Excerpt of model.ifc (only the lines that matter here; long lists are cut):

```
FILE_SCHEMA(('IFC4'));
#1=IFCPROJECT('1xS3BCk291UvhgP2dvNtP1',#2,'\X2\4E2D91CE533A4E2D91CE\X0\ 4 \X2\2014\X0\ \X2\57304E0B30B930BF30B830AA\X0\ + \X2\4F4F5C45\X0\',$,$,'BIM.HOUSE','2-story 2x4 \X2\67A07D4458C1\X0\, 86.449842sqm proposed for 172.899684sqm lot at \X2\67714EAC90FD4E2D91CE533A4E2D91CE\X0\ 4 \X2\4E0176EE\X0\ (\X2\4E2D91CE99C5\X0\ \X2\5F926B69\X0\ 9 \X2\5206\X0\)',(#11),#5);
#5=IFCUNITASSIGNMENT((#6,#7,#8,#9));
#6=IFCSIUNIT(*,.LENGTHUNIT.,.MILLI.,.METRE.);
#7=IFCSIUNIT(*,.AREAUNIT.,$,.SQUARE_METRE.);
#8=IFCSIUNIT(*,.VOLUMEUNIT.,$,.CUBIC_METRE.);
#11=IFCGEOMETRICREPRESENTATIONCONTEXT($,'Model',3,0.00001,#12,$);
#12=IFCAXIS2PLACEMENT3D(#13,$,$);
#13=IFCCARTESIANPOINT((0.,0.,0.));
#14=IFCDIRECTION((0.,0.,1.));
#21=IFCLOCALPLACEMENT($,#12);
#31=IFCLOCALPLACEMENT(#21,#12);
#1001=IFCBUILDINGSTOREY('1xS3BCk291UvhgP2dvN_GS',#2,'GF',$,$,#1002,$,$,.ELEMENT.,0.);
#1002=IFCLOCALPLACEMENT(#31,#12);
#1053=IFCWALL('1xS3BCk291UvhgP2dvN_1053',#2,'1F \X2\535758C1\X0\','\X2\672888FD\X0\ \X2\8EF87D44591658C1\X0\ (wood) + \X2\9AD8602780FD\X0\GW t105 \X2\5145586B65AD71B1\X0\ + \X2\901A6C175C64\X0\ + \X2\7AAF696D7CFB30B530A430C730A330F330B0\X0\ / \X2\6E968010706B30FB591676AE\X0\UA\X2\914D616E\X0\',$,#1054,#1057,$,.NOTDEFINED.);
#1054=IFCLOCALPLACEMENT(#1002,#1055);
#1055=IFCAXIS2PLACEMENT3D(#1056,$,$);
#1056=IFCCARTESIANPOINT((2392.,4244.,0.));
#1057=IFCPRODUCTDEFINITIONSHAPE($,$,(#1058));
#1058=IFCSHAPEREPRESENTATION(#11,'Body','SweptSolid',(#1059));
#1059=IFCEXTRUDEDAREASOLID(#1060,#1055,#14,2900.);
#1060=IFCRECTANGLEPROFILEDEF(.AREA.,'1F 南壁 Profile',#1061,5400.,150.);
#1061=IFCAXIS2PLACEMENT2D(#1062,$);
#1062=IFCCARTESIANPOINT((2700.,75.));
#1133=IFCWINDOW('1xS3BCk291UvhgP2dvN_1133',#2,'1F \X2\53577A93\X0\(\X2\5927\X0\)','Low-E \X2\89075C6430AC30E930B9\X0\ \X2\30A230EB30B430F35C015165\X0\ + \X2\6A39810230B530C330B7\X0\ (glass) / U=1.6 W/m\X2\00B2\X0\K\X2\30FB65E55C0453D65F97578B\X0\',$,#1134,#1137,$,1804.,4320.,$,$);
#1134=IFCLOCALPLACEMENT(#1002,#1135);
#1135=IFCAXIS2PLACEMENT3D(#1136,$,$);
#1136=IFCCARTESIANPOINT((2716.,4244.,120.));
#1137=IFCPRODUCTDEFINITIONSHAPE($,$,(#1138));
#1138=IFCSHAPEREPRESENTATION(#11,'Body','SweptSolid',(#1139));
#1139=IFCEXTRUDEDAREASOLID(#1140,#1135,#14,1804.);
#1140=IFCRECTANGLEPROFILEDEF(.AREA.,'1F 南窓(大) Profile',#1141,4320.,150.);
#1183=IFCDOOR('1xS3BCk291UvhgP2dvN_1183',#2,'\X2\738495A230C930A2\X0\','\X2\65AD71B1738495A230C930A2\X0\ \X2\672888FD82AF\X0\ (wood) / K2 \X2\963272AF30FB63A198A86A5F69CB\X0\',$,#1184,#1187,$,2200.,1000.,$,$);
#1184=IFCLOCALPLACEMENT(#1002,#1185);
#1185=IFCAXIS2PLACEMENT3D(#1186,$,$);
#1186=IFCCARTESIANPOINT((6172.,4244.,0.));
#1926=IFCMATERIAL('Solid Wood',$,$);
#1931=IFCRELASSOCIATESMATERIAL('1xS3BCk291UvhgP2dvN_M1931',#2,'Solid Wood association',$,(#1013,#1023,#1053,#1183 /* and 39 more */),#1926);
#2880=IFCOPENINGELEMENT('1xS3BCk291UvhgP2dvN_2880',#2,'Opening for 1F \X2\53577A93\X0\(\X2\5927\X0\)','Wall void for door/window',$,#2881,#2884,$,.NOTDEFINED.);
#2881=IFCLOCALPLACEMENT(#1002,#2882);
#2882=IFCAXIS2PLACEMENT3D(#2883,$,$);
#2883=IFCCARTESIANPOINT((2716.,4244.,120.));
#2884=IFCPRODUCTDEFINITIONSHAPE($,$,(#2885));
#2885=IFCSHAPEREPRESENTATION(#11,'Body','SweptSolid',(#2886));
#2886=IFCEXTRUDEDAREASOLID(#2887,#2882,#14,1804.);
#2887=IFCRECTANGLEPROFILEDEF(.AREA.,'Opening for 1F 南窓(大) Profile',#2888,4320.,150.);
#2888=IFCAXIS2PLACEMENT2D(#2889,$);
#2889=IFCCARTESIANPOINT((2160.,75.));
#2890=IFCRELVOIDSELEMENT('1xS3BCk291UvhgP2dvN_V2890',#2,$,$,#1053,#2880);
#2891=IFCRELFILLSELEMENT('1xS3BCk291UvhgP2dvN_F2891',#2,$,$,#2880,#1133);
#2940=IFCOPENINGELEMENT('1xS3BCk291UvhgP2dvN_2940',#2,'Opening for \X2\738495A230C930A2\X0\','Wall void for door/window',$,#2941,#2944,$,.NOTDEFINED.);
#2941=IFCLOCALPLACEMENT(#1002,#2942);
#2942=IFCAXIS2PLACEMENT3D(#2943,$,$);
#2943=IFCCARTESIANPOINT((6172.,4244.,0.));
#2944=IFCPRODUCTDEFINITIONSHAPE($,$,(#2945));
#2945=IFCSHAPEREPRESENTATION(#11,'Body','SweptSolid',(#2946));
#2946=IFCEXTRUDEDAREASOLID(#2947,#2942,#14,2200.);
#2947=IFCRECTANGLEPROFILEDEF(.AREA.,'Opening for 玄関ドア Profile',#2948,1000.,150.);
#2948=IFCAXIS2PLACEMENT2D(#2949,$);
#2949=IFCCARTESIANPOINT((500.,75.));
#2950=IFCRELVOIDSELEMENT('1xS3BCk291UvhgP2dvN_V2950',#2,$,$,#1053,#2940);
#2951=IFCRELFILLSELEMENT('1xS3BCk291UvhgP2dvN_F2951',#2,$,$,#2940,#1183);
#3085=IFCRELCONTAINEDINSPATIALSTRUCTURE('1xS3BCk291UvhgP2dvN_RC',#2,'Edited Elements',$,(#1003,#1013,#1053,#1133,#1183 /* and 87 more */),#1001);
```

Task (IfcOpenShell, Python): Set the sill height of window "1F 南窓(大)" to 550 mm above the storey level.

```python
import numpy as np
import ifcopenshell
import ifcopenshell.api.geometry
import ifcopenshell.geom
import ifcopenshell.util.element
import ifcopenshell.util.placement
import ifcopenshell.util.shape
import ifcopenshell.util.unit

model = ifcopenshell.open("model.ifc")
unit_scale = ifcopenshell.util.unit.calculate_unit_scale(model)

window = model.by_guid("1xS3BCk291UvhgP2dvN_1133")
opening = window.FillsVoids[0].RelatingOpeningElement
storey = ifcopenshell.util.element.get_container(window, ifc_class="IfcBuildingStorey")
level = ifcopenshell.util.placement.get_local_placement(storey.ObjectPlacement)[2, 3]

# The opening's origin need not be at the sill, so measure its lowest point.
shape = ifcopenshell.geom.create_shape(ifcopenshell.geom.settings(), opening)
bottom = ifcopenshell.util.shape.get_shape_bottom_elevation(shape, shape.geometry) / unit_scale
dz = level + 550.0 - bottom

shift = np.array([0.0, 0.0, dz])
# The window is not placed relative to its opening, so move both.
for product in (opening, window):
    matrix = ifcopenshell.util.placement.get_local_placement(product.ObjectPlacement)
    matrix[:3, 3] += shift
    ifcopenshell.api.geometry.edit_object_placement(model, product=product, matrix=matrix, is_si=False)

print(f"moved by {dz * unit_scale:+.3f} m")

model.write("model_rev.ifc")
```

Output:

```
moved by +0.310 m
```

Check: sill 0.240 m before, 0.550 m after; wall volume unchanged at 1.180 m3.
